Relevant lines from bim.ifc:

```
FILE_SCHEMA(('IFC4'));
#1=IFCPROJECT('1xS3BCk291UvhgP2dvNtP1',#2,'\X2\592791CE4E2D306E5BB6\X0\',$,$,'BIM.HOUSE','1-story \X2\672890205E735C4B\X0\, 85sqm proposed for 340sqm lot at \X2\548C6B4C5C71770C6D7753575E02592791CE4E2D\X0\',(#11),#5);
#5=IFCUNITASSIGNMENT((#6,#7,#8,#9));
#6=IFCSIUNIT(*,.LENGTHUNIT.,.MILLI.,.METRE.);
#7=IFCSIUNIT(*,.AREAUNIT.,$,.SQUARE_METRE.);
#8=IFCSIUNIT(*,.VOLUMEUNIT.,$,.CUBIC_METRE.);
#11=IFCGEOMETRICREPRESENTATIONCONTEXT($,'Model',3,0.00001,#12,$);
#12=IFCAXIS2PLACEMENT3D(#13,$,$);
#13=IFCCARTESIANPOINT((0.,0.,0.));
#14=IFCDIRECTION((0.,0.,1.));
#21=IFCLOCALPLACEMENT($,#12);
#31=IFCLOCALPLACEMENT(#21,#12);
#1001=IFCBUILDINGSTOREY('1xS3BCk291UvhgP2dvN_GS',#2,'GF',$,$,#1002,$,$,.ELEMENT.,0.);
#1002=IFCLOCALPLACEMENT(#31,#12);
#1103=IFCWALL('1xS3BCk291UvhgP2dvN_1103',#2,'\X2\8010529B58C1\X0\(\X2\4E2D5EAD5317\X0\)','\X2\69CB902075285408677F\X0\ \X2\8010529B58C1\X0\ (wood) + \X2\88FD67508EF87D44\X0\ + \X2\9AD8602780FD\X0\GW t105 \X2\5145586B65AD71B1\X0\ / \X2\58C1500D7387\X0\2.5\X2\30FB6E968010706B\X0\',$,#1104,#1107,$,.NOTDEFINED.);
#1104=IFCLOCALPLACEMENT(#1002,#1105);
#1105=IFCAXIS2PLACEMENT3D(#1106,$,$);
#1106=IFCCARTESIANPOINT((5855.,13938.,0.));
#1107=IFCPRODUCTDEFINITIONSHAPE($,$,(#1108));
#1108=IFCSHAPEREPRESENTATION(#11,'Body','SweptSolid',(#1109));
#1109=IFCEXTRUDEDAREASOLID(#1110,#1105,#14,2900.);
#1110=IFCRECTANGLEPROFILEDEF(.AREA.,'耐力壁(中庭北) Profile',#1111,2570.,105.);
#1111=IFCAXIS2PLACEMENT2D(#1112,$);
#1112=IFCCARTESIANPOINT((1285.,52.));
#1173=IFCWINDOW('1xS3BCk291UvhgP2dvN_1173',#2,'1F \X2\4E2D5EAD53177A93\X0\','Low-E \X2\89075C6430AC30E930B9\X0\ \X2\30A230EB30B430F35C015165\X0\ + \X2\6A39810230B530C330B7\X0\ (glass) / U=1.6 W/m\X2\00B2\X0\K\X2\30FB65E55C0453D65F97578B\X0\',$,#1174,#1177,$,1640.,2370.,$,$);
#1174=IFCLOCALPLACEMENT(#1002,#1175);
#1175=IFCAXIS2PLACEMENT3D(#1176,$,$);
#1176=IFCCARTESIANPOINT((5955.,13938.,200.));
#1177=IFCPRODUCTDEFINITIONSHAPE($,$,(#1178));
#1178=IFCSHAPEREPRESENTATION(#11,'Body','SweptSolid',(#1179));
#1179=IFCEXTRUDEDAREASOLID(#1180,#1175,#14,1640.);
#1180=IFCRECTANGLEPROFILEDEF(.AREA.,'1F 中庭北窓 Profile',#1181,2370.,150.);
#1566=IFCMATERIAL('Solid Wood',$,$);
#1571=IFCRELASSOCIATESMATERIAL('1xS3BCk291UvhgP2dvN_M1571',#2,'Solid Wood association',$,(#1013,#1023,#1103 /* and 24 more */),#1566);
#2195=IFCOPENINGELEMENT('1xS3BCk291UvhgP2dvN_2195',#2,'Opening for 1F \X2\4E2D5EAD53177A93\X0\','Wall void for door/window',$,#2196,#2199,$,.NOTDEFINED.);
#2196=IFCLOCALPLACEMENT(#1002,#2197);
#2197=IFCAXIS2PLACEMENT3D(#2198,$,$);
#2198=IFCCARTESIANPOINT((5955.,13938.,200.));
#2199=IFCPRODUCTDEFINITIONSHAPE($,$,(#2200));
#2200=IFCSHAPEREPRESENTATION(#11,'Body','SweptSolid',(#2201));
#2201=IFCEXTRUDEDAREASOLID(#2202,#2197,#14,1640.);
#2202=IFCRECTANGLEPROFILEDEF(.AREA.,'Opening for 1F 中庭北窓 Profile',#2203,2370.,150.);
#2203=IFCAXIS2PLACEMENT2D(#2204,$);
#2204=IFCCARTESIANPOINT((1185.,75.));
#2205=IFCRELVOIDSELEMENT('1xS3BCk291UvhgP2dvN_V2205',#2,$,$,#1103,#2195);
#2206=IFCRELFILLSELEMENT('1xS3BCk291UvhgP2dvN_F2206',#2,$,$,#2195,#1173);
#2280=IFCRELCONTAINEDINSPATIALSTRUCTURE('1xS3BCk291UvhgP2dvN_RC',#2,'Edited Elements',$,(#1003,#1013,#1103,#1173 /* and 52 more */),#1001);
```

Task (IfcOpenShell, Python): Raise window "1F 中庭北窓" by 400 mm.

```python
import numpy as np
import ifcopenshell
import ifcopenshell.api.geometry
import ifcopenshell.util.placement
import ifcopenshell.util.unit

model = ifcopenshell.open("bim.ifc")
unit_scale = ifcopenshell.util.unit.calculate_unit_scale(model)

window = model.by_id(1173)
opening = window.FillsVoids[0].RelatingOpeningElement
dz = 400.0

shift = np.array([0.0, 0.0, dz])
# The window is not placed relative to its opening, so move both.
for product in (opening, window):
    matrix = ifcopenshell.util.placement.get_local_placement(product.ObjectPlacement)
    matrix[:3, 3] += shift
    ifcopenshell.api.geometry.edit_object_placement(model, product=product, matrix=matrix, is_si=False)

print(f"moved by {dz * unit_scale:+.3f} m")

model.write("bim-out.ifc")
```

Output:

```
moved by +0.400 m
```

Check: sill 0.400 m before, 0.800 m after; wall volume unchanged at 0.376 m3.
